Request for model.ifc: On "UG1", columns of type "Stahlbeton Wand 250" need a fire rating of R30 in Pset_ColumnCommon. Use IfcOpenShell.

First a look at what the model holds.

```python
import ifcopenshell
import ifcopenshell.util.element

model = ifcopenshell.open("model.ifc")
print(model.schema)
storey = next(s for s in model.by_type("IfcBuildingStorey") if s.Name == "UG1")
columns = [e for e in ifcopenshell.util.element.get_decomposition(storey) if e.is_a("IfcColumn")]
seen = {}
for e in columns:
    element_type = ifcopenshell.util.element.get_type(e)
    key = (element_type.Name if element_type != e and element_type else None, ifcopenshell.util.element.get_pset(e, "Pset_ColumnCommon", "FireRating"))
    seen[key] = seen.get(key, 0) + 1
for (name, value), count in sorted(seen.items(), key=str):
    print(count, "x", name, "|", value)
```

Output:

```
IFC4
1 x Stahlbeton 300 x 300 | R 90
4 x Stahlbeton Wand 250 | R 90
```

```python
import ifcopenshell
import ifcopenshell.api.pset
import ifcopenshell.util.element

model = ifcopenshell.open("model.ifc")

storey = next(s for s in model.by_type("IfcBuildingStorey") if s.Name == "UG1")
columns = [e for e in ifcopenshell.util.element.get_decomposition(storey) if e.is_a("IfcColumn")]

count = 0
for e in columns:
    element_type = ifcopenshell.util.element.get_type(e)
    if element_type in (None, e) or element_type.Name != "Stahlbeton Wand 250":
        continue
    # add_pset returns the element's existing set when there is one.
    pset = ifcopenshell.api.pset.add_pset(model, product=e, name="Pset_ColumnCommon")
    ifcopenshell.api.pset.edit_pset(model, pset=pset, properties={"FireRating": "R30"})
    count += 1

print(count, "columns updated")

model.write("model-out.ifc")
```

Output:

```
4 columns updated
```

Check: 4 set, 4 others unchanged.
